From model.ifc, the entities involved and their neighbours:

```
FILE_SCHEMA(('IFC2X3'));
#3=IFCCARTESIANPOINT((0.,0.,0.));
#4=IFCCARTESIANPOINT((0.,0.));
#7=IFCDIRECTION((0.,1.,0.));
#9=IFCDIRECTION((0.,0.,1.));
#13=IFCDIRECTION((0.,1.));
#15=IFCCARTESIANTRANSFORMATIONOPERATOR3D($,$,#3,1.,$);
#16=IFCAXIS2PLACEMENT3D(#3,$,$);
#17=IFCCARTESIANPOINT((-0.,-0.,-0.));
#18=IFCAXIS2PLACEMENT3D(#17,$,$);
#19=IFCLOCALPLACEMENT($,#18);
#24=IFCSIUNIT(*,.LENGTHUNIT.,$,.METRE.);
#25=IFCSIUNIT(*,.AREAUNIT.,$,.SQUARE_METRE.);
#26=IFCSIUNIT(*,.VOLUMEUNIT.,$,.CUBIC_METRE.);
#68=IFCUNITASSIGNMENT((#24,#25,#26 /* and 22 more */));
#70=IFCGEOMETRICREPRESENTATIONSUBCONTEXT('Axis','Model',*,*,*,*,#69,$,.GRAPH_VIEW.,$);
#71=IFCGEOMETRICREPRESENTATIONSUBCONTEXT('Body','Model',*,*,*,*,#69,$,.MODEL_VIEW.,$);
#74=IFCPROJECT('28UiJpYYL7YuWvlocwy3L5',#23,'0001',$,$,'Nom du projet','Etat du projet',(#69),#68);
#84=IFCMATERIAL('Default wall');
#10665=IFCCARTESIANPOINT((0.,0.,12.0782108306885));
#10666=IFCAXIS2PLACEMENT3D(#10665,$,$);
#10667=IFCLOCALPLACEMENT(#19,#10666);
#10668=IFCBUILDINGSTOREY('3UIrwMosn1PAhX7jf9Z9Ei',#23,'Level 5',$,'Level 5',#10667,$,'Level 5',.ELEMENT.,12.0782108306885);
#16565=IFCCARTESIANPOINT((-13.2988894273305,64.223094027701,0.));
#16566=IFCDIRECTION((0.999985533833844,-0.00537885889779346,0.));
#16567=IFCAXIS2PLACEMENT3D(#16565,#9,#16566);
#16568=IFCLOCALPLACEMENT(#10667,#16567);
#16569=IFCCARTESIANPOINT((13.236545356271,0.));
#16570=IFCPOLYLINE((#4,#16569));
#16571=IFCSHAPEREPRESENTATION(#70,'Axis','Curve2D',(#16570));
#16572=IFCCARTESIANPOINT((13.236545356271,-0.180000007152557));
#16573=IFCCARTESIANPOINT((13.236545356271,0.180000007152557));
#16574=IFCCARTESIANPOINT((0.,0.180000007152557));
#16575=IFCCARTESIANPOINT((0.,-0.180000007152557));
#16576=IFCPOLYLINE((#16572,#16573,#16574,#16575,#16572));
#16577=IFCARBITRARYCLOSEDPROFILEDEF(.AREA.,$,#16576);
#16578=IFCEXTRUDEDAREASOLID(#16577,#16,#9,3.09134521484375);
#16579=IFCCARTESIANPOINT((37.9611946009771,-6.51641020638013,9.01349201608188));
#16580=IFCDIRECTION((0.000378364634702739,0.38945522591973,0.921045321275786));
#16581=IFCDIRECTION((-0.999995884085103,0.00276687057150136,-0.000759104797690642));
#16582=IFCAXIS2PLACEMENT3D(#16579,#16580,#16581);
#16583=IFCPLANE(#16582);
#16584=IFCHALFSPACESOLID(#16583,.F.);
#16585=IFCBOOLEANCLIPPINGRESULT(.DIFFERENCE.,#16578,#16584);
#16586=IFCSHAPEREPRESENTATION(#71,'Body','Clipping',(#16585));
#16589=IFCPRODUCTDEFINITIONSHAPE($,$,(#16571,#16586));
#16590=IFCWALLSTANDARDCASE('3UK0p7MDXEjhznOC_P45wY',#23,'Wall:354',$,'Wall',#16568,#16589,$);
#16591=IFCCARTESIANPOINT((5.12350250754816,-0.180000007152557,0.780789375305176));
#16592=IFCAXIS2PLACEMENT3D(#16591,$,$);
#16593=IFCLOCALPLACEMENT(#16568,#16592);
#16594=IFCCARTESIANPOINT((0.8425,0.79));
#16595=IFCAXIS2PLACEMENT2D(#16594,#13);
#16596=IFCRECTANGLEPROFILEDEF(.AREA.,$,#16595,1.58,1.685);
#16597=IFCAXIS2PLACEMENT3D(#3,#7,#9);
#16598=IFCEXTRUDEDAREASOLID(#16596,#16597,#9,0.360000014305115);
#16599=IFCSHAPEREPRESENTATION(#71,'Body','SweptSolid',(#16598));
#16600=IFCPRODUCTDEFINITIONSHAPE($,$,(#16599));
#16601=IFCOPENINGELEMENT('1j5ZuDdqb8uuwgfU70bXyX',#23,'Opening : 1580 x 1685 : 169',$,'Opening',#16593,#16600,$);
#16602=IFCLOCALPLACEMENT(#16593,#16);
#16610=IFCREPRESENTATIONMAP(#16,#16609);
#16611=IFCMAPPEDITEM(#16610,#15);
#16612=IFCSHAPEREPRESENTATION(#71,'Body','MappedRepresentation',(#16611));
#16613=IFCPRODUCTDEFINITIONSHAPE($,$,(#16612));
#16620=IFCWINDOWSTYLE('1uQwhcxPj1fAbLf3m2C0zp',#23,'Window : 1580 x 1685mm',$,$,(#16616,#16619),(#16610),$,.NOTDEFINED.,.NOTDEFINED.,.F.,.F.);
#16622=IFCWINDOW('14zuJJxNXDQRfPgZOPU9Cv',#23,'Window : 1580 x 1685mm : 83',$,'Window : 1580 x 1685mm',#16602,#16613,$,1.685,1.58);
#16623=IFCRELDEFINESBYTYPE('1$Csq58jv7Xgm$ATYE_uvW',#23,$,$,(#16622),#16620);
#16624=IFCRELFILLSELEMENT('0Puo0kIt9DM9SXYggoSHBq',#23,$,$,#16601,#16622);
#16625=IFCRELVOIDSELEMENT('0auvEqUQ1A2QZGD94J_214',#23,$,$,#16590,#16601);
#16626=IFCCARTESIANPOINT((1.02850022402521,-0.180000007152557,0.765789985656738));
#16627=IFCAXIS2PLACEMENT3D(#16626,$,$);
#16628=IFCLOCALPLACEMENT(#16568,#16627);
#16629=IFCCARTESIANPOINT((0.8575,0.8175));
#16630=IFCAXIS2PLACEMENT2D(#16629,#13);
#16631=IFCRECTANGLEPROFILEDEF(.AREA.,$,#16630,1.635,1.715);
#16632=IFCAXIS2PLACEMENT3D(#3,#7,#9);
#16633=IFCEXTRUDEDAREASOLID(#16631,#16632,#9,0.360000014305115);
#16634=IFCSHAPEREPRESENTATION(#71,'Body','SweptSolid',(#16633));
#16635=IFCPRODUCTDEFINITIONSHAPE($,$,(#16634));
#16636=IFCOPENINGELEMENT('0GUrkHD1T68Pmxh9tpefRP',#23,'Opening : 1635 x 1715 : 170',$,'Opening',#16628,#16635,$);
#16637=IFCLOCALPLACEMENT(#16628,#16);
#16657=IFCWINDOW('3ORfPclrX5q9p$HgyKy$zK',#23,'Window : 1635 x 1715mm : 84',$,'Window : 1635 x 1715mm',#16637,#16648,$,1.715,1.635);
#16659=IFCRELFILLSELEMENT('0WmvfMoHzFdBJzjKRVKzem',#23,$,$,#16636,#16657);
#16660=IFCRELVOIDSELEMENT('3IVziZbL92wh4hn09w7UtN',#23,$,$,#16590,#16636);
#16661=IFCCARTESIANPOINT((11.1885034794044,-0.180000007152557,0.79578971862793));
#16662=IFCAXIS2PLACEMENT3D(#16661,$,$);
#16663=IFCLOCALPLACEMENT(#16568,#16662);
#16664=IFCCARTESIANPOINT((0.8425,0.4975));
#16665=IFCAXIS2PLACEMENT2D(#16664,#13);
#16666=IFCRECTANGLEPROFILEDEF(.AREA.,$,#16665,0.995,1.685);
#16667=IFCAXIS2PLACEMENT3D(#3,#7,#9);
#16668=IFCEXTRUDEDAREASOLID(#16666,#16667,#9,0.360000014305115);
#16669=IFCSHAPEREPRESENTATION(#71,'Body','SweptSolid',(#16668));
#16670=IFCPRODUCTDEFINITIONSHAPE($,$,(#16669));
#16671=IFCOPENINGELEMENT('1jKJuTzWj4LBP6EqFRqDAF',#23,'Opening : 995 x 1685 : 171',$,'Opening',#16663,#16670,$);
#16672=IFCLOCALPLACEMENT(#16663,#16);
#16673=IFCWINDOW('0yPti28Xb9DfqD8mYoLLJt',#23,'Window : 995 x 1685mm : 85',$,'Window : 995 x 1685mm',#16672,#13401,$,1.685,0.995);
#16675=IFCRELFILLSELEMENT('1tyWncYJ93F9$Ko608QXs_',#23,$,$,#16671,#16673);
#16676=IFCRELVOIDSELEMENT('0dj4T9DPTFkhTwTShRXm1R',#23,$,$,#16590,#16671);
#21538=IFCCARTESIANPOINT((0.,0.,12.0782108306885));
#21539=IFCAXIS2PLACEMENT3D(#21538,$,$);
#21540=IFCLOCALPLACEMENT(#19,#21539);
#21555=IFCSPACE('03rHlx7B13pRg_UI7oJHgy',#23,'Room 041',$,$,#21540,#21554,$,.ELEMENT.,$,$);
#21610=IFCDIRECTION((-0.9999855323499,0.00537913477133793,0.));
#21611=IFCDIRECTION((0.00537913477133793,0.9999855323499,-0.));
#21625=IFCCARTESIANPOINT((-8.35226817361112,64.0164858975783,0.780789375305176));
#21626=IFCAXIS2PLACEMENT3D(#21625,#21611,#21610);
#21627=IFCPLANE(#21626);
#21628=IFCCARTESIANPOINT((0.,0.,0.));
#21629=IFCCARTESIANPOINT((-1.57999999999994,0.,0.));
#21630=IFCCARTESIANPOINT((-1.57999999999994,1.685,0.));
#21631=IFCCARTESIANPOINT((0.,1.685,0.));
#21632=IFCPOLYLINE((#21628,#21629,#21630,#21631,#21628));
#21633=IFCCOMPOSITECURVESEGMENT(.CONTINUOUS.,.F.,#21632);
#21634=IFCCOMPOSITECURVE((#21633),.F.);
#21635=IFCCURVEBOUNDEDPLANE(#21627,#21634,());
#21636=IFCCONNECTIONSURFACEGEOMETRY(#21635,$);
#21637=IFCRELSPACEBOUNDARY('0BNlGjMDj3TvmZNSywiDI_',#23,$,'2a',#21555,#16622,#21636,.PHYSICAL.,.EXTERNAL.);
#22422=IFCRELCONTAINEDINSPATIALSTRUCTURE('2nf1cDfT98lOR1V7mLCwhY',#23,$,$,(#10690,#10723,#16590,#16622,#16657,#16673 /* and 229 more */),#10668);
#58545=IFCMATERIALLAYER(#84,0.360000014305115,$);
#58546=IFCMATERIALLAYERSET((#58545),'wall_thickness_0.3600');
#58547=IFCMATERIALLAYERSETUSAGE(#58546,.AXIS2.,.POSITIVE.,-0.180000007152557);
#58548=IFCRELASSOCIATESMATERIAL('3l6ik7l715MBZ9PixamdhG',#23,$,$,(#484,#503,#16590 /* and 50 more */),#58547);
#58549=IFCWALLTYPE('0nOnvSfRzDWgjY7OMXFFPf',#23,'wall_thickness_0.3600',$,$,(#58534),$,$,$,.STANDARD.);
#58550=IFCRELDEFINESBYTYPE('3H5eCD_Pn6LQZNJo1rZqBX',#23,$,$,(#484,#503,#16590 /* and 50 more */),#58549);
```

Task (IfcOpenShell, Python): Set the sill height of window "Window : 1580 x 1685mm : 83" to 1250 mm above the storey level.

```python
import numpy as np
import ifcopenshell
import ifcopenshell.api.geometry
import ifcopenshell.geom
import ifcopenshell.util.element
import ifcopenshell.util.placement
import ifcopenshell.util.shape
import ifcopenshell.util.unit

model = ifcopenshell.open("model.ifc")
unit_scale = ifcopenshell.util.unit.calculate_unit_scale(model)

window = model.by_guid("14zuJJxNXDQRfPgZOPU9Cv")
opening = window.FillsVoids[0].RelatingOpeningElement
storey = ifcopenshell.util.element.get_container(window, ifc_class="IfcBuildingStorey")
level = ifcopenshell.util.placement.get_local_placement(storey.ObjectPlacement)[2, 3]

# The opening's origin need not be at the sill, so measure its lowest point.
shape = ifcopenshell.geom.create_shape(ifcopenshell.geom.settings(), opening)
bottom = ifcopenshell.util.shape.get_shape_bottom_elevation(shape, shape.geometry) / unit_scale
dz = level + 1.25 / unit_scale - bottom

shift = np.array([0.0, 0.0, dz])
# The window is placed relative to its opening, so it follows when the opening moves.
matrix = ifcopenshell.util.placement.get_local_placement(opening.ObjectPlacement)
matrix[:3, 3] += shift
ifcopenshell.api.geometry.edit_object_placement(
    model, product=opening, matrix=matrix, is_si=False, should_transform_children=True
)

# Space boundary surfaces are stored in each space's coordinates; move them too.
for rel in window.ProvidesBoundaries:
    if not rel.ConnectionGeometry:
        continue
    surface = rel.ConnectionGeometry.SurfaceOnRelatingElement.BasisSurface
    space_matrix = ifcopenshell.util.placement.get_local_placement(rel.RelatingSpace.ObjectPlacement)
    point = np.array(surface.Position.Location.Coordinates) + space_matrix[:3, :3].T @ shift
    surface.Position = model.createIfcAxis2Placement3D(
        model.createIfcCartesianPoint(point.tolist()), surface.Position.Axis, surface.Position.RefDirection
    )

print(f"moved by {dz * unit_scale:+.3f} m")

model.write("model_v2.ifc")
```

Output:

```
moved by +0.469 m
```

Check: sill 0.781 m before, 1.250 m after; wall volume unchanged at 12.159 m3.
